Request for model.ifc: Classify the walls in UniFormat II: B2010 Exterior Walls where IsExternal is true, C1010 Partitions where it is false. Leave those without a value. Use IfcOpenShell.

First a look at what the model holds.

```python
import ifcopenshell
import ifcopenshell.util.element

model = ifcopenshell.open("model.ifc")
print(model.schema)
print("classifications:", [c.Name for c in model.by_type("IfcClassification")])
values = [ifcopenshell.util.element.get_pset(e, "Pset_WallCommon", "IsExternal") for e in model.by_type("IfcWall")]
for value in (True, False, None):
    print("IsExternal", value, values.count(value))
```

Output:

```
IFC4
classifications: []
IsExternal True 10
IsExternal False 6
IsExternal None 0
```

```python
import ifcopenshell
import ifcopenshell.api.classification
import ifcopenshell.util.element

model = ifcopenshell.open("model.ifc")

system = ifcopenshell.api.classification.add_classification(model, classification="UniFormat II")

walls = model.by_type("IfcWall")
external = {e: ifcopenshell.util.element.get_pset(e, "Pset_WallCommon", "IsExternal") for e in walls}
for flag, code, name in ((True, "B2010", "Exterior Walls"), (False, "C1010", "Partitions")):
    products = [e for e in walls if external[e] is flag]
    ifcopenshell.api.classification.add_reference(
        model, products=products, classification=system, identification=code, name=name
    )
    print(code, len(products))

model.write("model_updated.ifc")
```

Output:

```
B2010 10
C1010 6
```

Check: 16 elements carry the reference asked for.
